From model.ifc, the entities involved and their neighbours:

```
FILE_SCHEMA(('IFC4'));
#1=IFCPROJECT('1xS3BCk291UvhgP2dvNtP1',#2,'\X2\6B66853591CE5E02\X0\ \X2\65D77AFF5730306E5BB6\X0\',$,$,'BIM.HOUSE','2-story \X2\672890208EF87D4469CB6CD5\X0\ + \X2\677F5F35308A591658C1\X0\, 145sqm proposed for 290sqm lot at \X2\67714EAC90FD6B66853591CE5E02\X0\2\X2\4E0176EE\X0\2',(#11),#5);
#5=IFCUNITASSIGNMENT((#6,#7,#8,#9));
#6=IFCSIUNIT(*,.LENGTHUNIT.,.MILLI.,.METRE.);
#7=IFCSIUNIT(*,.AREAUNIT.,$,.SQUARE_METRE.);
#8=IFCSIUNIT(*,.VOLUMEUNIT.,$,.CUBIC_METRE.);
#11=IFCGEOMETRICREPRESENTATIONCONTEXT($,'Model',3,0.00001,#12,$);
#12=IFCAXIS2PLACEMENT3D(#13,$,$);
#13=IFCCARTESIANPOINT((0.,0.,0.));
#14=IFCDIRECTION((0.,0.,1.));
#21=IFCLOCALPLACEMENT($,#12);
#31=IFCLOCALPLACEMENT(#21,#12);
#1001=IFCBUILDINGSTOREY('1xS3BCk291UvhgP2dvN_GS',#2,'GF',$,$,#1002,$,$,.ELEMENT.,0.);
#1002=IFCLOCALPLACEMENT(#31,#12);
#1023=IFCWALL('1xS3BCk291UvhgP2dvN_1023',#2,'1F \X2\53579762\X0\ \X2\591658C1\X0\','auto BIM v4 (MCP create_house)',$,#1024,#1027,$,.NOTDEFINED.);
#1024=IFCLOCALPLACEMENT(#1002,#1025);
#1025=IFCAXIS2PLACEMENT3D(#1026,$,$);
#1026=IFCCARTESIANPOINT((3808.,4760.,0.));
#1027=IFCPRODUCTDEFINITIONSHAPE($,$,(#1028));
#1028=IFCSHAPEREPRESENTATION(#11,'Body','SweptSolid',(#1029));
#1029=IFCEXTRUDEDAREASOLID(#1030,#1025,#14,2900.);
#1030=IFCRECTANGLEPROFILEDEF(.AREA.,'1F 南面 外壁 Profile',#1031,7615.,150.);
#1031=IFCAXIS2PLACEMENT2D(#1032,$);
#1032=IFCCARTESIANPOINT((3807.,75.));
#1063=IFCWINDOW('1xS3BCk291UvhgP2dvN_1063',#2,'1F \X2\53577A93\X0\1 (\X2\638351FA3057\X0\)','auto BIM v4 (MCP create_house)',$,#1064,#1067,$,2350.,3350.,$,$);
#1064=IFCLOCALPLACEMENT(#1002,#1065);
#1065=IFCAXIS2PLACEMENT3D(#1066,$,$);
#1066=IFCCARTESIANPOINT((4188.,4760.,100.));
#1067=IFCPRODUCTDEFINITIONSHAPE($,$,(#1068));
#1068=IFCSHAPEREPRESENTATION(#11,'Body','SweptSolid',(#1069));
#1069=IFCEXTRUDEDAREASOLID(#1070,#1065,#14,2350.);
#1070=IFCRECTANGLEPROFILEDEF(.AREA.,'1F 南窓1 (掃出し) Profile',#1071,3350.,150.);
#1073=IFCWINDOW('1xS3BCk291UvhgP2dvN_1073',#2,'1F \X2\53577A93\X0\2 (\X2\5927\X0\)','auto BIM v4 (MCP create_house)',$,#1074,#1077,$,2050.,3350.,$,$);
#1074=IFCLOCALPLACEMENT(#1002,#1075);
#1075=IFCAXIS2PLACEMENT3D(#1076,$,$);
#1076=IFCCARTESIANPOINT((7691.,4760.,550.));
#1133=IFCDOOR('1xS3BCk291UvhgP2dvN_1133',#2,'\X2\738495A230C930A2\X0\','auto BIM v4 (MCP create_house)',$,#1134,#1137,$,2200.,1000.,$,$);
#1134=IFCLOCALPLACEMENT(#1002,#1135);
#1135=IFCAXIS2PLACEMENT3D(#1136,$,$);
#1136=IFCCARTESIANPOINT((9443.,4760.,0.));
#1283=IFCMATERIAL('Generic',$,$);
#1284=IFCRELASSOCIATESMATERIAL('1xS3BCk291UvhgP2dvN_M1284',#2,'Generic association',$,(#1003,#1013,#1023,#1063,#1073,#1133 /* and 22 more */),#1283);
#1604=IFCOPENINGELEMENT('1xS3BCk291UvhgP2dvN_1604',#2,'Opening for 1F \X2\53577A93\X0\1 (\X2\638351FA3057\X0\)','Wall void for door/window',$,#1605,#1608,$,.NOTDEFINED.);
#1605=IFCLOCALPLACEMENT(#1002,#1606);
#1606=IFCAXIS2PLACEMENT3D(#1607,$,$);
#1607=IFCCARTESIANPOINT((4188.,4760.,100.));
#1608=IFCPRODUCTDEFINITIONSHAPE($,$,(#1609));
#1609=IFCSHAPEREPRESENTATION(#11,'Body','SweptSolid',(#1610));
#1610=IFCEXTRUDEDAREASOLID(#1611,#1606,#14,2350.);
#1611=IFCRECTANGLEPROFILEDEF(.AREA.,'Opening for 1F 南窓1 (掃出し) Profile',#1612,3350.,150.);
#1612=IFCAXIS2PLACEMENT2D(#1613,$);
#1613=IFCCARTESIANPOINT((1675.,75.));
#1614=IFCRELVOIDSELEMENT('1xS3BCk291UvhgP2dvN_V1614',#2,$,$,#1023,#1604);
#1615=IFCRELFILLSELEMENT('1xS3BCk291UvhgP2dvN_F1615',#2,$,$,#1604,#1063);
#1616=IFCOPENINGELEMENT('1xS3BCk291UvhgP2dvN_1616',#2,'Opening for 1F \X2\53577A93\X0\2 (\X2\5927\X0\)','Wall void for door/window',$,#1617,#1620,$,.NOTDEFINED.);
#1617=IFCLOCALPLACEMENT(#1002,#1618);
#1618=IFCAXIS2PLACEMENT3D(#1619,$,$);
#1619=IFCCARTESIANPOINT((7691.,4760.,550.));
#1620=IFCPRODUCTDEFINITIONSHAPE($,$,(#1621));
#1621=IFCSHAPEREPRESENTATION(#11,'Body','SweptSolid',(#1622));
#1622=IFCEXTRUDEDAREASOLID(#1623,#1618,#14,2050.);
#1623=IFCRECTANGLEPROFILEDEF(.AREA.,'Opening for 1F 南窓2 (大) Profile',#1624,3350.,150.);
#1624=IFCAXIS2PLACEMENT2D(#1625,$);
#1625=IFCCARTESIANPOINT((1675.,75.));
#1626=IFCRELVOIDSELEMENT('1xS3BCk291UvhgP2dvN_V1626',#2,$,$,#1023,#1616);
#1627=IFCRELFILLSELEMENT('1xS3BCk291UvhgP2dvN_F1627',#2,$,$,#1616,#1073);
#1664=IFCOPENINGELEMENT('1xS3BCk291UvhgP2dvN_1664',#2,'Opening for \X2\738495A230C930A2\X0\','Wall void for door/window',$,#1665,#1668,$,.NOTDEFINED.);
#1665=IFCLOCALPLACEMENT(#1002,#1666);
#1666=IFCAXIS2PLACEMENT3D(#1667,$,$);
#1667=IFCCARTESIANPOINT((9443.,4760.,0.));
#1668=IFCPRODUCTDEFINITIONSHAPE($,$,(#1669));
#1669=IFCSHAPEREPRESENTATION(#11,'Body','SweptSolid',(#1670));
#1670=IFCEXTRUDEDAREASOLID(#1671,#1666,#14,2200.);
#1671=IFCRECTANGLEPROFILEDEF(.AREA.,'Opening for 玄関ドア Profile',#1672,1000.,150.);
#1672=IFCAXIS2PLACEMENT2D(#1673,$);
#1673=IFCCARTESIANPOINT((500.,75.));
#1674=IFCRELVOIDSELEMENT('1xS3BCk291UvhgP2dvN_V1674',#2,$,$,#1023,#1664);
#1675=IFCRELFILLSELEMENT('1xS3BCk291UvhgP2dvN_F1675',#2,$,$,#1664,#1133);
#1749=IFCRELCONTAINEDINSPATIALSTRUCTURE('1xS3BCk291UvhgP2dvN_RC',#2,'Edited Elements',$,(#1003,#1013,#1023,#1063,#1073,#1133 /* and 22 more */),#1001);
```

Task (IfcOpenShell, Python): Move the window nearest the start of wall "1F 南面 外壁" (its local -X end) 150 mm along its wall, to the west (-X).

```python
import ifcopenshell
import ifcopenshell.api.geometry
import ifcopenshell.util.placement
import ifcopenshell.util.unit

model = ifcopenshell.open("model.ifc")
unit_scale = ifcopenshell.util.unit.calculate_unit_scale(model)

window = model.by_id(1063)
opening = window.FillsVoids[0].RelatingOpeningElement
wall = opening.VoidsElements[0].RelatingBuildingElement

wall_matrix = ifcopenshell.util.placement.get_local_placement(wall.ObjectPlacement)
shift = wall_matrix[:3, 0] * -0.15 / unit_scale
before = ifcopenshell.util.placement.get_local_placement(window.ObjectPlacement)[:3, 3].copy()

# The window is not placed relative to its opening, so move both.
for product in (opening, window):
    matrix = ifcopenshell.util.placement.get_local_placement(product.ObjectPlacement)
    matrix[:3, 3] += shift
    ifcopenshell.api.geometry.edit_object_placement(model, product=product, matrix=matrix, is_si=False)

after = ifcopenshell.util.placement.get_local_placement(window.ObjectPlacement)[:3, 3]
print("window moved by", (after - before).round(3) + 0.0)

model.write("model_edited.ifc")
```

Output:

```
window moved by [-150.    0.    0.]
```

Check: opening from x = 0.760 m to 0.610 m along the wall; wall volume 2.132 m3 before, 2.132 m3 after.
